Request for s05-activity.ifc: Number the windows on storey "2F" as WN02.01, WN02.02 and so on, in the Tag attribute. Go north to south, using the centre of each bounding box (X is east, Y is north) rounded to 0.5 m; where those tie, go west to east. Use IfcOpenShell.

First a look at what the model holds.

```python
import ifcopenshell
import ifcopenshell.util.element
import ifcopenshell.util.placement

model = ifcopenshell.open("s05-activity.ifc")
print(model.schema)
storey = next(s for s in model.by_type("IfcBuildingStorey") if s.Name == "2F")
windows = [e for e in ifcopenshell.util.element.get_decomposition(storey) if e.is_a("IfcWindow")]
for e in sorted(windows, key=lambda e: e.id()):
    origin = ifcopenshell.util.placement.get_local_placement(e.ObjectPlacement)[:3, 3]
    print(e.id(), e.Tag, e.Name, origin.round(2) + 0.0, sep=" | ")
```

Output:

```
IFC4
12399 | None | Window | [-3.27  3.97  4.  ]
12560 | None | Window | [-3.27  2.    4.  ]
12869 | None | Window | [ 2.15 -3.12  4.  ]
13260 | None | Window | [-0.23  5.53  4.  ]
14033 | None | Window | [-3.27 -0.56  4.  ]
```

```python
import ifcopenshell
import ifcopenshell.geom
import ifcopenshell.util.element
import ifcopenshell.util.shape

model = ifcopenshell.open("s05-activity.ifc")
settings = ifcopenshell.geom.settings()
settings.set("use-world-coords", True)


def centre(element):
    shape = ifcopenshell.geom.create_shape(settings, element)
    return ifcopenshell.util.shape.get_bbox_centroid(shape.geometry)


storey = next(s for s in model.by_type("IfcBuildingStorey") if s.Name == "2F")
windows = [e for e in ifcopenshell.util.element.get_decomposition(storey) if e.is_a("IfcWindow")]

# Insertion points can sit at a corner or the storey origin, so sort by the geometry (in metres).
centres = {e: centre(e) for e in windows}
windows.sort(key=lambda e: (-round(centres[e][1] / 0.5), centres[e][0]))

for i, e in enumerate(windows, start=1):
    number = f"WN02.{i:02d}"
    e.Tag = number
    print(e.id(), number)

model.write("s05-activity-out.ifc")
```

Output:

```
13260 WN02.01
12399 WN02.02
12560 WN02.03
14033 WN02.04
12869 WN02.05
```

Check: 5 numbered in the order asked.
